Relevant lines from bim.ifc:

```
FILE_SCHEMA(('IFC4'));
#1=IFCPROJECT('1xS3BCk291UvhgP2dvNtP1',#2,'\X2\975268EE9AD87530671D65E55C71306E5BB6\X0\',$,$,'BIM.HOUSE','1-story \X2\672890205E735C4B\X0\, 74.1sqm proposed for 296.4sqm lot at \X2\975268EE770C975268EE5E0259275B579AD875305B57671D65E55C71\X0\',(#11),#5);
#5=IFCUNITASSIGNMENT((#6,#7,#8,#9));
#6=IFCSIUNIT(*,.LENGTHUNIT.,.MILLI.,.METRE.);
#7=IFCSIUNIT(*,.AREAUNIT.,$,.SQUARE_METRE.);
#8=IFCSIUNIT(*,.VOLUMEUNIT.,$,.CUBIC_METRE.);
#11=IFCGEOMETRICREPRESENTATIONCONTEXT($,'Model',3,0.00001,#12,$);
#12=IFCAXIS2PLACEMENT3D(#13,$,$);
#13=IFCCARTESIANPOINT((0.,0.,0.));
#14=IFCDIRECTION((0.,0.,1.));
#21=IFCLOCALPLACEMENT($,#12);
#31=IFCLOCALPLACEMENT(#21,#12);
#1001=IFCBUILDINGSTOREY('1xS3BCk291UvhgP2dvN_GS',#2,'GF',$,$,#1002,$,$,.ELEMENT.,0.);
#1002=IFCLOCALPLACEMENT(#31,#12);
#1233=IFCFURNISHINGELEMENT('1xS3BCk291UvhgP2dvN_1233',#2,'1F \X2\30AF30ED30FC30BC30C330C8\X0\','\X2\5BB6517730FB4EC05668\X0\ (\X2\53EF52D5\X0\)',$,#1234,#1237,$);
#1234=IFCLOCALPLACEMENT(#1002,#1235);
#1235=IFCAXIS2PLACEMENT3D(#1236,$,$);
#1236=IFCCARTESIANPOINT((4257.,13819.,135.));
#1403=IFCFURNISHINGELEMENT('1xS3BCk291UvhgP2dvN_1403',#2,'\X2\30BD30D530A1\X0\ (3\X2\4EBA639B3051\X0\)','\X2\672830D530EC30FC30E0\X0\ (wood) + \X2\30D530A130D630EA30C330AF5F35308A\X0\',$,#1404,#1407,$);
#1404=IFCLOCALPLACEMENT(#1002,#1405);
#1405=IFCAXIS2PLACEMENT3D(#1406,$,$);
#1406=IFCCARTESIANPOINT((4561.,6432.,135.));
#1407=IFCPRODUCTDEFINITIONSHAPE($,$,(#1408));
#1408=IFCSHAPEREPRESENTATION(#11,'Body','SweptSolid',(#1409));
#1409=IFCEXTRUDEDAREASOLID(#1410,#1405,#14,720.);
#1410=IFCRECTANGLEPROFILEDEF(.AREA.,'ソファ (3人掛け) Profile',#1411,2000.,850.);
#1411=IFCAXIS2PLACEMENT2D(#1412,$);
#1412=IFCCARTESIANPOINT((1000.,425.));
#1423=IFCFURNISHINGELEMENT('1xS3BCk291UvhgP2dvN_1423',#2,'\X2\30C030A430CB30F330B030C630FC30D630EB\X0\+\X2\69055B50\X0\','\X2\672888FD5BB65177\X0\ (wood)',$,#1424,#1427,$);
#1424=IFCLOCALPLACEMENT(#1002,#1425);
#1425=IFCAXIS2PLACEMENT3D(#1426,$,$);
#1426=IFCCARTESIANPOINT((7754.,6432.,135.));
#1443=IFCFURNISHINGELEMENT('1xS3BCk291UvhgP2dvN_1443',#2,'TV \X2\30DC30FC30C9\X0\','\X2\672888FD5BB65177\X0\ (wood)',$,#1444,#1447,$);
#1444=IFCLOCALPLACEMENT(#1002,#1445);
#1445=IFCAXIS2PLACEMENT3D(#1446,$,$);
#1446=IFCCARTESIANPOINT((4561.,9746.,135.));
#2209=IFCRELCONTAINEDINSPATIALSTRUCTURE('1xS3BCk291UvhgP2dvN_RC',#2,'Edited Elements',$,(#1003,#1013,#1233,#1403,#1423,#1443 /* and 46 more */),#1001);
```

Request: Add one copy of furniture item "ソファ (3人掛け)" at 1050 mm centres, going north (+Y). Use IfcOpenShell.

```python
import numpy as np
import ifcopenshell
import ifcopenshell.api.geometry
import ifcopenshell.api.root
import ifcopenshell.util.element
import ifcopenshell.util.placement

model = ifcopenshell.open("bim.ifc")


def reuse_history(source, copy):
    """copy_class also copies each property set's owner history, people and application; keep the originals."""
    for rel in copy.IsDefinedBy:
        if rel.is_a("IfcRelDefinesByProperties") and (history := rel.RelatingPropertyDefinition.OwnerHistory):
            rel.RelatingPropertyDefinition.OwnerHistory = source.OwnerHistory
            ifcopenshell.util.element.remove_deep2(model, history)


source = model.by_guid("1xS3BCk291UvhgP2dvN_1403")
base = ifcopenshell.util.placement.get_local_placement(source.ObjectPlacement)
step = np.array([0.0, 1.0, 0.0]) * 1050.0

for i in range(1, 2):
    copy = ifcopenshell.api.root.copy_class(model, product=source)
    copy.Representation = ifcopenshell.util.element.copy_deep(
        model, source.Representation, exclude=["IfcGeometricRepresentationContext", "IfcRepresentationMap"]
    )
    reuse_history(source, copy)
    matrix = base.copy()
    matrix[:3, 3] += i * step
    print("added at", matrix[:3, 3].round(3) + 0.0)
    ifcopenshell.api.geometry.edit_object_placement(model, product=copy, matrix=matrix, is_si=False)

model.write("bim-out.ifc")
```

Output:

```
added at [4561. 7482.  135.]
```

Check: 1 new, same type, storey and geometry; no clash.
